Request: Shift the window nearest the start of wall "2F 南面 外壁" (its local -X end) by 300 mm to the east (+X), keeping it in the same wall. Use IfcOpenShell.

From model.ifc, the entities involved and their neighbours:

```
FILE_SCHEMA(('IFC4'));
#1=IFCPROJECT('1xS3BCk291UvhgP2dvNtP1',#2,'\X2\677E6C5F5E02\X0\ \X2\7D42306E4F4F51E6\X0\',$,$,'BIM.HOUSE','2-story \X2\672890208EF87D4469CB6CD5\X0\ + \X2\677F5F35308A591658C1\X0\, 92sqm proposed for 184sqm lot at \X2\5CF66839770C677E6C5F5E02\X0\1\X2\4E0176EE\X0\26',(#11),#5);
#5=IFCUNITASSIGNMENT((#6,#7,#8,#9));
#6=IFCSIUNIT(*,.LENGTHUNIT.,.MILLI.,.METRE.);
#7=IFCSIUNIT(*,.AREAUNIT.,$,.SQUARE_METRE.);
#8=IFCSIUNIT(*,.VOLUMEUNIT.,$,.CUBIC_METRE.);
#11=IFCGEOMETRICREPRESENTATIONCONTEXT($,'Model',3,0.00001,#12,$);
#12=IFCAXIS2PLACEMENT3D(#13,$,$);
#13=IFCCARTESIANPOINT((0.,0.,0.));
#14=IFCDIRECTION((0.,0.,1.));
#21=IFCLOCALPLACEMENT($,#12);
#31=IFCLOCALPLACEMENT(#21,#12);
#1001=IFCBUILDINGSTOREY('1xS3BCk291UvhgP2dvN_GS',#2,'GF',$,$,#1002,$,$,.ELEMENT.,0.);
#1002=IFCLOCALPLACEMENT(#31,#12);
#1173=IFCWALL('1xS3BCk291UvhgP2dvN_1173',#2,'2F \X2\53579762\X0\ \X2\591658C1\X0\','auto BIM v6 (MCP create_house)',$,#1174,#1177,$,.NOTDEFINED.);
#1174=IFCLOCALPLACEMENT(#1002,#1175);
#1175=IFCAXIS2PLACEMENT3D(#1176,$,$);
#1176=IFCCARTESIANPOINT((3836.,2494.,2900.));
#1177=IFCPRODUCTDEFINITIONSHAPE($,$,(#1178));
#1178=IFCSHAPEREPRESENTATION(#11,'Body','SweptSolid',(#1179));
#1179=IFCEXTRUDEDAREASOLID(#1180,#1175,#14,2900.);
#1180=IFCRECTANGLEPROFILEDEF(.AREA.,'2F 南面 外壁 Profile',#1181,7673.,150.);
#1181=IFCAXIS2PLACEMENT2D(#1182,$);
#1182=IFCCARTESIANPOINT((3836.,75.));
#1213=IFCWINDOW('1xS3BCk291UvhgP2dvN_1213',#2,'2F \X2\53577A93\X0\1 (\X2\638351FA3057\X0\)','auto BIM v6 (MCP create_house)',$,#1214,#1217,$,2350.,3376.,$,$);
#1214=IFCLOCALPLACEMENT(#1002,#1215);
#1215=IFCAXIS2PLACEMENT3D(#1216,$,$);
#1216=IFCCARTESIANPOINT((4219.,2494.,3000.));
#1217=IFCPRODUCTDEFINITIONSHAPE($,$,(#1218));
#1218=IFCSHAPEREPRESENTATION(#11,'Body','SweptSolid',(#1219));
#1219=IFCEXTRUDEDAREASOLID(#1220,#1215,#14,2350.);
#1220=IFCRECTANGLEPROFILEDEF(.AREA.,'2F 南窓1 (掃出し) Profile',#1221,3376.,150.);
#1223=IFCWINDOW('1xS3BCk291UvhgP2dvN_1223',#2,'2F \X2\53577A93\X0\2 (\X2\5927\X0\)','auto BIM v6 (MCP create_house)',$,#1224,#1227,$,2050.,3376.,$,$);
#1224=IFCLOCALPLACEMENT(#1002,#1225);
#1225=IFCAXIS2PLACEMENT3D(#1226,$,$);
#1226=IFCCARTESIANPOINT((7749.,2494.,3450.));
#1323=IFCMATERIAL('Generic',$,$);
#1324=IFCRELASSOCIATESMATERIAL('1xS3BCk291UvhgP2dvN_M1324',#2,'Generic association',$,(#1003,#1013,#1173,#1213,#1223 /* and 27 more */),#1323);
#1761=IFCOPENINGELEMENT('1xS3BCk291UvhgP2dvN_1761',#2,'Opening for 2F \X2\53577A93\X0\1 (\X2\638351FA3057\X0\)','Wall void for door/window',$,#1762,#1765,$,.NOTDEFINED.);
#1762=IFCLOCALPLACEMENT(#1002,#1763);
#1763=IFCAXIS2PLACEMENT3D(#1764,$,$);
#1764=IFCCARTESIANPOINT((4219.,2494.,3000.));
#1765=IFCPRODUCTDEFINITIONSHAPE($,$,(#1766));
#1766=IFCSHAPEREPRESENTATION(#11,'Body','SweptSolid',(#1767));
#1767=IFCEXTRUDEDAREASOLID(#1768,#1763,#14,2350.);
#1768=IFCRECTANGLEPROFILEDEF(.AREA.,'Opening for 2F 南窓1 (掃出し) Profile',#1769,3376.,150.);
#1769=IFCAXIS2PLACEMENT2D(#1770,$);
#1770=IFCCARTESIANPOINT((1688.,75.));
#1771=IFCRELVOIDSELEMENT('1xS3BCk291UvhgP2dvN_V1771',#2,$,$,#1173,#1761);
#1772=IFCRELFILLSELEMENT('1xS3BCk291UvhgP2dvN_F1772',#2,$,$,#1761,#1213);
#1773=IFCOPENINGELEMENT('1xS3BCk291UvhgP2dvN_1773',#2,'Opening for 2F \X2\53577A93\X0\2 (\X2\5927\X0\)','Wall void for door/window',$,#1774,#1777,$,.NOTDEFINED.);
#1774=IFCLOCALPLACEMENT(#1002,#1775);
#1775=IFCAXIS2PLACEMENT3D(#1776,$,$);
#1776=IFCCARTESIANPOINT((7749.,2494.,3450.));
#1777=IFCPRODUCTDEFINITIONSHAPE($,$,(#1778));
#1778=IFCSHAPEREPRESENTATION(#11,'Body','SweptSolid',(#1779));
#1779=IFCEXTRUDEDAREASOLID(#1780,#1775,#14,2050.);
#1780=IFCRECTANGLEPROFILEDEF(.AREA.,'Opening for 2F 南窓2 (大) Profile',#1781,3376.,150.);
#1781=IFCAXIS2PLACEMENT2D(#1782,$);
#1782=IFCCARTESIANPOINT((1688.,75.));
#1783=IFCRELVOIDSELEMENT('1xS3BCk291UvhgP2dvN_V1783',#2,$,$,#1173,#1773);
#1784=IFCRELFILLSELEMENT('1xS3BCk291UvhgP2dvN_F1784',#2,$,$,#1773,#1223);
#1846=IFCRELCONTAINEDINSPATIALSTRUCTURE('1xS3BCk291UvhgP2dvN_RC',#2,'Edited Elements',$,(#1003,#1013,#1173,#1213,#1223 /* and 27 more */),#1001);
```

```python
import ifcopenshell
import ifcopenshell.api.geometry
import ifcopenshell.util.placement
import ifcopenshell.util.unit

model = ifcopenshell.open("model.ifc")
unit_scale = ifcopenshell.util.unit.calculate_unit_scale(model)

window = model.by_guid("1xS3BCk291UvhgP2dvN_1213")
opening = window.FillsVoids[0].RelatingOpeningElement
wall = opening.VoidsElements[0].RelatingBuildingElement

wall_matrix = ifcopenshell.util.placement.get_local_placement(wall.ObjectPlacement)
shift = wall_matrix[:3, 0] * 0.3 / unit_scale
before = ifcopenshell.util.placement.get_local_placement(window.ObjectPlacement)[:3, 3].copy()

# The window is not placed relative to its opening, so move both.
for product in (opening, window):
    matrix = ifcopenshell.util.placement.get_local_placement(product.ObjectPlacement)
    matrix[:3, 3] += shift
    ifcopenshell.api.geometry.edit_object_placement(model, product=product, matrix=matrix, is_si=False)

after = ifcopenshell.util.placement.get_local_placement(window.ObjectPlacement)[:3, 3]
print("window moved by", (after - before).round(3) + 0.0)

model.write("model_rev.ifc")
```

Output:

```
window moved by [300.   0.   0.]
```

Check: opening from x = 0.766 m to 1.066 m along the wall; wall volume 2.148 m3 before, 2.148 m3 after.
